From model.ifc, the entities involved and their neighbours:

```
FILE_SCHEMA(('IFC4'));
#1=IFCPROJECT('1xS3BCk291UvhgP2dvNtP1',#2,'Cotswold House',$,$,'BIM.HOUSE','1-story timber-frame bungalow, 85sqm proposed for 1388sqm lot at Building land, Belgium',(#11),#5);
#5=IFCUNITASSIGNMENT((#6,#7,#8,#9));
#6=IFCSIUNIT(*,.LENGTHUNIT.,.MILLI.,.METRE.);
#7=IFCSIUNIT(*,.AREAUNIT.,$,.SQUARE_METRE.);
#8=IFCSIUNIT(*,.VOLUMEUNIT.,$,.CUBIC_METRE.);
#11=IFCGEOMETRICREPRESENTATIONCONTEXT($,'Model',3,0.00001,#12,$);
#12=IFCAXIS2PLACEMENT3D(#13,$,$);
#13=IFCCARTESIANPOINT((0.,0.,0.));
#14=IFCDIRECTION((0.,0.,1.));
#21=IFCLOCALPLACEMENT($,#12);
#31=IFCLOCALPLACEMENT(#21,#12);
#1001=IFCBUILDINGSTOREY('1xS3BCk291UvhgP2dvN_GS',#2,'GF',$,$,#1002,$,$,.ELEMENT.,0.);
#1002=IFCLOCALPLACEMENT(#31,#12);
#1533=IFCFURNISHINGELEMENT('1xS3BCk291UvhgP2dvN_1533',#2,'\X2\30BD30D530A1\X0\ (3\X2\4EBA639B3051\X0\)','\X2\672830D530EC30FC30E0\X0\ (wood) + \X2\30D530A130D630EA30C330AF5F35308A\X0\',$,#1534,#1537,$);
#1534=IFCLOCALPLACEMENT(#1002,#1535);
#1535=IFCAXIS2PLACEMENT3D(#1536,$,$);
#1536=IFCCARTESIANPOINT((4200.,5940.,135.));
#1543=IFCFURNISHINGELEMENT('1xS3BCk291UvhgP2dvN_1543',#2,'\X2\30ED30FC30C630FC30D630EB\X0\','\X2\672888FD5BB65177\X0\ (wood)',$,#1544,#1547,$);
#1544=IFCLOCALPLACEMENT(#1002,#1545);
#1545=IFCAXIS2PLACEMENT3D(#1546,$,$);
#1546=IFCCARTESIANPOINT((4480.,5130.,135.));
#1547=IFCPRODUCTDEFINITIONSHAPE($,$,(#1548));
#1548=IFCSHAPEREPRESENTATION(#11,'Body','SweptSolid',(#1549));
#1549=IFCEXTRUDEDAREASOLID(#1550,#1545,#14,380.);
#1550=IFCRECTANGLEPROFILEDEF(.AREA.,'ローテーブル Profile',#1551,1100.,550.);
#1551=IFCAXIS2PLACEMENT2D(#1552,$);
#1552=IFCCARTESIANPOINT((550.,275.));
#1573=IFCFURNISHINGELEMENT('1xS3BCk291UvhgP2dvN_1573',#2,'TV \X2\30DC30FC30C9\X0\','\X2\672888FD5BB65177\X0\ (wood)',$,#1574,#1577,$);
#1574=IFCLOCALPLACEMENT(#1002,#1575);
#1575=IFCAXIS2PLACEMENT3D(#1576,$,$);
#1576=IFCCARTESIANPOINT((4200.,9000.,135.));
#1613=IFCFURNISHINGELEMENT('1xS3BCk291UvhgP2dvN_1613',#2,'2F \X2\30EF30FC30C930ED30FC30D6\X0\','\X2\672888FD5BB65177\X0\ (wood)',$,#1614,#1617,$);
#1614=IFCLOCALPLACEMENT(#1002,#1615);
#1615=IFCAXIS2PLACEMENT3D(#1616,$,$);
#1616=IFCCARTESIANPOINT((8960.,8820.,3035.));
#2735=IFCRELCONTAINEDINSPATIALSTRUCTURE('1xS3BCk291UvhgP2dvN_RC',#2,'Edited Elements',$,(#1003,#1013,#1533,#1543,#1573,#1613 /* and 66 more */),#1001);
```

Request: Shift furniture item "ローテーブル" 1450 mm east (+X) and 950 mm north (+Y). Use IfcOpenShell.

```python
import ifcopenshell
import ifcopenshell.api.geometry
import ifcopenshell.util.placement
import ifcopenshell.util.unit

model = ifcopenshell.open("model.ifc")
unit_scale = ifcopenshell.util.unit.calculate_unit_scale(model)

item = model.by_guid("1xS3BCk291UvhgP2dvN_1543")
matrix = ifcopenshell.util.placement.get_local_placement(item.ObjectPlacement)
matrix[0, 3] += 1.45 / unit_scale
matrix[1, 3] += 0.95 / unit_scale
ifcopenshell.api.geometry.edit_object_placement(model, product=item, matrix=matrix, is_si=False)

print(ifcopenshell.util.placement.get_local_placement(item.ObjectPlacement).round(3) + 0.0)

model.write("model_edited.ifc")
```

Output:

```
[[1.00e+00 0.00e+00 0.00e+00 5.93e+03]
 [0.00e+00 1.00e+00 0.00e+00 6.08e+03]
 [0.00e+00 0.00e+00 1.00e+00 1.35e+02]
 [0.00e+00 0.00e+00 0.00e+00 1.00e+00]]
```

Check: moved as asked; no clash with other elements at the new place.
